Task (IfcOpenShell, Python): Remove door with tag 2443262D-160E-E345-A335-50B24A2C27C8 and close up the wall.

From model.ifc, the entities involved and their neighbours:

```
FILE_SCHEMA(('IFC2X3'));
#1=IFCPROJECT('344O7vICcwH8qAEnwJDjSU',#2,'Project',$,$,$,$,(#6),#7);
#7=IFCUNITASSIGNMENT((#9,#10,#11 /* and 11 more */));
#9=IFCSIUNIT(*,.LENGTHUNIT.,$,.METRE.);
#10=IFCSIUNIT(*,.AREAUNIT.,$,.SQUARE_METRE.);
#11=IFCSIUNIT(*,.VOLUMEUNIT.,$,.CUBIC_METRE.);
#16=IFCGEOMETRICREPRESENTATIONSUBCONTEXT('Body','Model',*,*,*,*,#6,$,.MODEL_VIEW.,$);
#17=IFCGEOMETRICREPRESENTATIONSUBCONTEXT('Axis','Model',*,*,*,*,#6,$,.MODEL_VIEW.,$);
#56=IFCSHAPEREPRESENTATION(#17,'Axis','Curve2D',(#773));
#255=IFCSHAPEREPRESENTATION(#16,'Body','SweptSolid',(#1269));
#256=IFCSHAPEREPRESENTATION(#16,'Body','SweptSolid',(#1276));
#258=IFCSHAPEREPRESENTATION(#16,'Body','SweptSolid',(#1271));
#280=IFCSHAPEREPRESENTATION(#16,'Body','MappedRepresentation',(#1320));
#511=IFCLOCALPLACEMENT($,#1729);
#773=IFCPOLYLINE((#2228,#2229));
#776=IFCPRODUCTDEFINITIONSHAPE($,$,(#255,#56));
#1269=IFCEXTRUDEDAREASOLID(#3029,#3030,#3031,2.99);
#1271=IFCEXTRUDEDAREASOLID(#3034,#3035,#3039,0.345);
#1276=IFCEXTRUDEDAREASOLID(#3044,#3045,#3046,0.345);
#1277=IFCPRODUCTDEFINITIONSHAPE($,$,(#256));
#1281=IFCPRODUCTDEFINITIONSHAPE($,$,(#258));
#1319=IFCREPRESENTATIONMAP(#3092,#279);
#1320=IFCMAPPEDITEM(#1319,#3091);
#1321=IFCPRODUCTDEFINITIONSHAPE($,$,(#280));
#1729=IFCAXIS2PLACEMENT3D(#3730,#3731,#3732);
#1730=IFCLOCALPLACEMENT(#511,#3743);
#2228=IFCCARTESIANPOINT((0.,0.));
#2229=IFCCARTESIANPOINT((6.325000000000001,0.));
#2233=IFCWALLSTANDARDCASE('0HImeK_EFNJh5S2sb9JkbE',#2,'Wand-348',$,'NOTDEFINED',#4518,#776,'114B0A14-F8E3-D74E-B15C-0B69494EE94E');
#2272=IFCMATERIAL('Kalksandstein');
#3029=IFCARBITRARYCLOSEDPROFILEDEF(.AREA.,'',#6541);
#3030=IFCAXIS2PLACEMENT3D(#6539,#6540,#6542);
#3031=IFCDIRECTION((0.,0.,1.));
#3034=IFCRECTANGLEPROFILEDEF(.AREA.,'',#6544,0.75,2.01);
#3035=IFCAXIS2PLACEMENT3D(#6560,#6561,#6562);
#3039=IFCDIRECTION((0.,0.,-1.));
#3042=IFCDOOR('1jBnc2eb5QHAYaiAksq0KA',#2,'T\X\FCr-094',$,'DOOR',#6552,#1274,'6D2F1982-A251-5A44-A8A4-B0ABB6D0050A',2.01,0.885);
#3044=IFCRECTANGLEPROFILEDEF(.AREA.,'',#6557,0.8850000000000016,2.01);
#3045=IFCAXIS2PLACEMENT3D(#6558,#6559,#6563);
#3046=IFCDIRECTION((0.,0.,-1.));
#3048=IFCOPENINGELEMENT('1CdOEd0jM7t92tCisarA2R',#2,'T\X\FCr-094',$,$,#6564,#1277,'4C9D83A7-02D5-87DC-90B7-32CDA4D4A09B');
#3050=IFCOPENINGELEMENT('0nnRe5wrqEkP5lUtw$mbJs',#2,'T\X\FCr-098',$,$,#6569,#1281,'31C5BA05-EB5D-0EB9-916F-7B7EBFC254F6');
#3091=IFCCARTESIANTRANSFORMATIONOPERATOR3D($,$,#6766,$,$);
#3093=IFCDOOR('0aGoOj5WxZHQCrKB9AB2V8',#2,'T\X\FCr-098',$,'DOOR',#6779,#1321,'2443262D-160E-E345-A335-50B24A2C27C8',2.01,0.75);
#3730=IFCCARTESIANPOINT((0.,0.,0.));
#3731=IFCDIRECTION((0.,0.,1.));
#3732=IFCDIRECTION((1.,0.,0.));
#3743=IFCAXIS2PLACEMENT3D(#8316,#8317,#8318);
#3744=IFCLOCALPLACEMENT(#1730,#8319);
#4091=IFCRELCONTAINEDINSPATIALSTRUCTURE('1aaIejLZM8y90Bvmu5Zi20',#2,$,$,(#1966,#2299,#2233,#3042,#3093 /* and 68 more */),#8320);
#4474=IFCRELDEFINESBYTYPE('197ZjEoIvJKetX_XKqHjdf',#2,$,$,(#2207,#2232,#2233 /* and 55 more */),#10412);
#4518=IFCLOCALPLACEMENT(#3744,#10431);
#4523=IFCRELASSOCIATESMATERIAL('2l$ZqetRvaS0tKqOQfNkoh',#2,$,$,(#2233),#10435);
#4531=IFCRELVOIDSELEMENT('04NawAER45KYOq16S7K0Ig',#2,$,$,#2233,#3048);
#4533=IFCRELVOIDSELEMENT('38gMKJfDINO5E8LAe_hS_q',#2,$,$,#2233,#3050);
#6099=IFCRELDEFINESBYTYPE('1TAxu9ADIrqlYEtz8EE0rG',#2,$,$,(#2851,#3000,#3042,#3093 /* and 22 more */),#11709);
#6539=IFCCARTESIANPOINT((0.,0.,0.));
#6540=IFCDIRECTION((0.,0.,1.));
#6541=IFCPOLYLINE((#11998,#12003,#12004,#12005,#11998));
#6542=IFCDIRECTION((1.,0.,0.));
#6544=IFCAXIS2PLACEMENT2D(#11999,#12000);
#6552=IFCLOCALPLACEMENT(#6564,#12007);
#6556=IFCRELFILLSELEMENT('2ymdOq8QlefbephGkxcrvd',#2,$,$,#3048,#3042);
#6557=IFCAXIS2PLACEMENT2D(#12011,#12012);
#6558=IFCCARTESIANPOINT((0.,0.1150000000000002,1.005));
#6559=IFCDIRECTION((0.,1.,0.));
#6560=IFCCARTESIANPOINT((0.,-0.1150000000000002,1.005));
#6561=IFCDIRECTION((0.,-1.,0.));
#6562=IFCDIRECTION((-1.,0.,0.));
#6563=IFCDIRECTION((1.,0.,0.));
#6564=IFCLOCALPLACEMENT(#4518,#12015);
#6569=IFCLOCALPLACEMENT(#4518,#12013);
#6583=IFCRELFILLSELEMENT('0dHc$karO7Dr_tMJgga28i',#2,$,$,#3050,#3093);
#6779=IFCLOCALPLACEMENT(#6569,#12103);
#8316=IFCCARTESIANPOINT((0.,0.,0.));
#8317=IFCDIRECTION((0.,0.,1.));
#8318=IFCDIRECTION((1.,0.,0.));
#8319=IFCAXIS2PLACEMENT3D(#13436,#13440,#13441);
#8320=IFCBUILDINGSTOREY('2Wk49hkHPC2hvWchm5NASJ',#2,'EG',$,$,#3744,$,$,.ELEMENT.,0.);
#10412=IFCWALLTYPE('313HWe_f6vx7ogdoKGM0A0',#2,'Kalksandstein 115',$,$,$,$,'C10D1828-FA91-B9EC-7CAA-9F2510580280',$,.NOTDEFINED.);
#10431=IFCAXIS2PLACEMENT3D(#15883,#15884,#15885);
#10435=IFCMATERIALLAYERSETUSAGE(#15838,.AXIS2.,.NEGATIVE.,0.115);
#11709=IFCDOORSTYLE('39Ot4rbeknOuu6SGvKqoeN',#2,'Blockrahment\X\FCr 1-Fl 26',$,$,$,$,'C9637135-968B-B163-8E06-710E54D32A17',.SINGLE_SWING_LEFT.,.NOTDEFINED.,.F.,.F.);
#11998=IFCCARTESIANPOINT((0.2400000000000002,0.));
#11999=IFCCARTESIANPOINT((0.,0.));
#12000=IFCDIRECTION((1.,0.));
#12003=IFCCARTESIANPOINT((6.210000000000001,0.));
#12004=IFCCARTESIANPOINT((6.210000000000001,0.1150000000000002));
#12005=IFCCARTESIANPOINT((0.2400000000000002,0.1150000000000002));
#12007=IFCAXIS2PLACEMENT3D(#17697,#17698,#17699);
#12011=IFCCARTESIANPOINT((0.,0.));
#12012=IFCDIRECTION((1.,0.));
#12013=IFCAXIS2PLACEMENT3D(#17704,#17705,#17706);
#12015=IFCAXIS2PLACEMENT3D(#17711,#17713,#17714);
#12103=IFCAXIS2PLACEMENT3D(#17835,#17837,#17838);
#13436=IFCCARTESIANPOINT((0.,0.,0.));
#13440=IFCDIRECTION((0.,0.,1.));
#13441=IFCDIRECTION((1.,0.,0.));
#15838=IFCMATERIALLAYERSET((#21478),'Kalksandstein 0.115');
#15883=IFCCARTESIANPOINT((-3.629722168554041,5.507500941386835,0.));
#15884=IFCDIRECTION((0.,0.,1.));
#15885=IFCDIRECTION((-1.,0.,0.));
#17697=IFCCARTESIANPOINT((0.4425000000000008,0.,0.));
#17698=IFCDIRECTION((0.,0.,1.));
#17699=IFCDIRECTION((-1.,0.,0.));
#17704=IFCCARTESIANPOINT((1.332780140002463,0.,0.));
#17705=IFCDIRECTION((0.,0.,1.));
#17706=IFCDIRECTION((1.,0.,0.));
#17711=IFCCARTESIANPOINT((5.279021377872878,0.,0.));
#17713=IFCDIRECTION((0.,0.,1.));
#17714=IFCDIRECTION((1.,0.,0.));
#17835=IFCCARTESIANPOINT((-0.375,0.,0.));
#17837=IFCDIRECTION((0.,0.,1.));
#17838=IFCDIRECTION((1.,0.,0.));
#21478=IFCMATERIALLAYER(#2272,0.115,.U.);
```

```python
import ifcopenshell
import ifcopenshell.api.feature
import ifcopenshell.api.root
import ifcopenshell.geom
import ifcopenshell.util.shape

model = ifcopenshell.open("model.ifc")
settings = ifcopenshell.geom.settings()


def volume(element):
    """Net volume in cubic metres, openings subtracted."""
    shape = ifcopenshell.geom.create_shape(settings, element)
    return ifcopenshell.util.shape.get_volume(shape.geometry)


door = model.by_id(3093)
opening = door.FillsVoids[0].RelatingOpeningElement
wall = opening.VoidsElements[0].RelatingBuildingElement
before = volume(wall)

ifcopenshell.api.root.remove_product(model, product=door)
ifcopenshell.api.feature.remove_feature(model, feature=opening)

after = volume(wall)

print(f"wall volume {before:.3f} -> {after:.3f} m3")

model.write("model_v2.ifc")
```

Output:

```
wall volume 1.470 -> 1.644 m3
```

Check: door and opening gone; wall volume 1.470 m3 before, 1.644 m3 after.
